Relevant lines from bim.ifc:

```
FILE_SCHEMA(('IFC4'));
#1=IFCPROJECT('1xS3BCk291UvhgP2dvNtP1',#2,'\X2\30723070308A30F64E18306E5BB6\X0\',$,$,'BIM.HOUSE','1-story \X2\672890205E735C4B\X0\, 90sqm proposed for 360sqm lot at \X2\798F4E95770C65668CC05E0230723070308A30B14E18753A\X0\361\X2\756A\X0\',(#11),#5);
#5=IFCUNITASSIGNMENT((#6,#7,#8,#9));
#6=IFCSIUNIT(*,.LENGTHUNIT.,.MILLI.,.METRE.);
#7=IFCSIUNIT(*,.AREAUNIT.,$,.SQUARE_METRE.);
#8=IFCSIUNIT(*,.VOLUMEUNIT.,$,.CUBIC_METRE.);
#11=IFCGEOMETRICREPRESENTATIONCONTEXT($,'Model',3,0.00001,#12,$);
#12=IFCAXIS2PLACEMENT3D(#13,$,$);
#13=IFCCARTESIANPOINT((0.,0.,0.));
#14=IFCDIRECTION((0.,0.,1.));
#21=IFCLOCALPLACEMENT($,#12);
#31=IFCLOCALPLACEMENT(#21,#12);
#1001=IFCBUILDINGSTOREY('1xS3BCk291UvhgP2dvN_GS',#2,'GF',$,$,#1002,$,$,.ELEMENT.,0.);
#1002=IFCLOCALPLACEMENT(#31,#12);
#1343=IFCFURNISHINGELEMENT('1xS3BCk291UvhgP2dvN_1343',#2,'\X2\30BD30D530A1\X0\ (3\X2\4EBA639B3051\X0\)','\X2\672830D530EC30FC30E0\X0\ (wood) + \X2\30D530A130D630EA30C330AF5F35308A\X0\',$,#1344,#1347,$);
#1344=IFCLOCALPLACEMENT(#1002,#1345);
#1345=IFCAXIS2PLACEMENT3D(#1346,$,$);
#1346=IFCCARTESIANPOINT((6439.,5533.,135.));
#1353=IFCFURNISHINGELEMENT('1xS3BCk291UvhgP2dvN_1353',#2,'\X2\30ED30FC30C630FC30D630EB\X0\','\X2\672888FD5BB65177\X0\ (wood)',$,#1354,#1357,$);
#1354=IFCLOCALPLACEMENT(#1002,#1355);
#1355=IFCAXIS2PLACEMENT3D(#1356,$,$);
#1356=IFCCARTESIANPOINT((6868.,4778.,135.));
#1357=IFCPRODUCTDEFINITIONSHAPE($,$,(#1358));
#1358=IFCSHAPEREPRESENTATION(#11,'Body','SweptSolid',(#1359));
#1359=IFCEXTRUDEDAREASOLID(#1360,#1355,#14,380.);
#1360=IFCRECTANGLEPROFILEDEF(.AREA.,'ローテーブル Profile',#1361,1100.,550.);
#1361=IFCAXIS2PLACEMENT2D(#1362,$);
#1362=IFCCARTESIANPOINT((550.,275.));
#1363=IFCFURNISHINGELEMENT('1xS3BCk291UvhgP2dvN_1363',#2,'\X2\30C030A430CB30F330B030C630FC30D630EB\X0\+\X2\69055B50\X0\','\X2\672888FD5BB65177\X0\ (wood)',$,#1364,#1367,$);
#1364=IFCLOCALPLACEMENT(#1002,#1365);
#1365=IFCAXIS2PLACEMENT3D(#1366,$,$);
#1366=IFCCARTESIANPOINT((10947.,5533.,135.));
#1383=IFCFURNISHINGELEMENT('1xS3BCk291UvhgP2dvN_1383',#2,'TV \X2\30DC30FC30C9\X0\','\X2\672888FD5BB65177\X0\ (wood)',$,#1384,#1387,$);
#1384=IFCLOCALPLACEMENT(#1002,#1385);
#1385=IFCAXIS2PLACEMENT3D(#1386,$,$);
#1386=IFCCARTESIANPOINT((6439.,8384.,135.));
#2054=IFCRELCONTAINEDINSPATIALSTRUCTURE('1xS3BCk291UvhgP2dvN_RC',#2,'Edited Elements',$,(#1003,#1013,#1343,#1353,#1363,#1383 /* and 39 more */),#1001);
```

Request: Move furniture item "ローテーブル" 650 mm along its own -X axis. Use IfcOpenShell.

```python
import ifcopenshell
import ifcopenshell.api.geometry
import ifcopenshell.util.placement
import ifcopenshell.util.unit

model = ifcopenshell.open("bim.ifc")
unit_scale = ifcopenshell.util.unit.calculate_unit_scale(model)

item = model.by_guid("1xS3BCk291UvhgP2dvN_1353")
matrix = ifcopenshell.util.placement.get_local_placement(item.ObjectPlacement)
matrix[:3, 3] -= matrix[:3, 0] * 0.65 / unit_scale
ifcopenshell.api.geometry.edit_object_placement(model, product=item, matrix=matrix, is_si=False)

print(ifcopenshell.util.placement.get_local_placement(item.ObjectPlacement).round(3) + 0.0)

model.write("bim-out.ifc")
```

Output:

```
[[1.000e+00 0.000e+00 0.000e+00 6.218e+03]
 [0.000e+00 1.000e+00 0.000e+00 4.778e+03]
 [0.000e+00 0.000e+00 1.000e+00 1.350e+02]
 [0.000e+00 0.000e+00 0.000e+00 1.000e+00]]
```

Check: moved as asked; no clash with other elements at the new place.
